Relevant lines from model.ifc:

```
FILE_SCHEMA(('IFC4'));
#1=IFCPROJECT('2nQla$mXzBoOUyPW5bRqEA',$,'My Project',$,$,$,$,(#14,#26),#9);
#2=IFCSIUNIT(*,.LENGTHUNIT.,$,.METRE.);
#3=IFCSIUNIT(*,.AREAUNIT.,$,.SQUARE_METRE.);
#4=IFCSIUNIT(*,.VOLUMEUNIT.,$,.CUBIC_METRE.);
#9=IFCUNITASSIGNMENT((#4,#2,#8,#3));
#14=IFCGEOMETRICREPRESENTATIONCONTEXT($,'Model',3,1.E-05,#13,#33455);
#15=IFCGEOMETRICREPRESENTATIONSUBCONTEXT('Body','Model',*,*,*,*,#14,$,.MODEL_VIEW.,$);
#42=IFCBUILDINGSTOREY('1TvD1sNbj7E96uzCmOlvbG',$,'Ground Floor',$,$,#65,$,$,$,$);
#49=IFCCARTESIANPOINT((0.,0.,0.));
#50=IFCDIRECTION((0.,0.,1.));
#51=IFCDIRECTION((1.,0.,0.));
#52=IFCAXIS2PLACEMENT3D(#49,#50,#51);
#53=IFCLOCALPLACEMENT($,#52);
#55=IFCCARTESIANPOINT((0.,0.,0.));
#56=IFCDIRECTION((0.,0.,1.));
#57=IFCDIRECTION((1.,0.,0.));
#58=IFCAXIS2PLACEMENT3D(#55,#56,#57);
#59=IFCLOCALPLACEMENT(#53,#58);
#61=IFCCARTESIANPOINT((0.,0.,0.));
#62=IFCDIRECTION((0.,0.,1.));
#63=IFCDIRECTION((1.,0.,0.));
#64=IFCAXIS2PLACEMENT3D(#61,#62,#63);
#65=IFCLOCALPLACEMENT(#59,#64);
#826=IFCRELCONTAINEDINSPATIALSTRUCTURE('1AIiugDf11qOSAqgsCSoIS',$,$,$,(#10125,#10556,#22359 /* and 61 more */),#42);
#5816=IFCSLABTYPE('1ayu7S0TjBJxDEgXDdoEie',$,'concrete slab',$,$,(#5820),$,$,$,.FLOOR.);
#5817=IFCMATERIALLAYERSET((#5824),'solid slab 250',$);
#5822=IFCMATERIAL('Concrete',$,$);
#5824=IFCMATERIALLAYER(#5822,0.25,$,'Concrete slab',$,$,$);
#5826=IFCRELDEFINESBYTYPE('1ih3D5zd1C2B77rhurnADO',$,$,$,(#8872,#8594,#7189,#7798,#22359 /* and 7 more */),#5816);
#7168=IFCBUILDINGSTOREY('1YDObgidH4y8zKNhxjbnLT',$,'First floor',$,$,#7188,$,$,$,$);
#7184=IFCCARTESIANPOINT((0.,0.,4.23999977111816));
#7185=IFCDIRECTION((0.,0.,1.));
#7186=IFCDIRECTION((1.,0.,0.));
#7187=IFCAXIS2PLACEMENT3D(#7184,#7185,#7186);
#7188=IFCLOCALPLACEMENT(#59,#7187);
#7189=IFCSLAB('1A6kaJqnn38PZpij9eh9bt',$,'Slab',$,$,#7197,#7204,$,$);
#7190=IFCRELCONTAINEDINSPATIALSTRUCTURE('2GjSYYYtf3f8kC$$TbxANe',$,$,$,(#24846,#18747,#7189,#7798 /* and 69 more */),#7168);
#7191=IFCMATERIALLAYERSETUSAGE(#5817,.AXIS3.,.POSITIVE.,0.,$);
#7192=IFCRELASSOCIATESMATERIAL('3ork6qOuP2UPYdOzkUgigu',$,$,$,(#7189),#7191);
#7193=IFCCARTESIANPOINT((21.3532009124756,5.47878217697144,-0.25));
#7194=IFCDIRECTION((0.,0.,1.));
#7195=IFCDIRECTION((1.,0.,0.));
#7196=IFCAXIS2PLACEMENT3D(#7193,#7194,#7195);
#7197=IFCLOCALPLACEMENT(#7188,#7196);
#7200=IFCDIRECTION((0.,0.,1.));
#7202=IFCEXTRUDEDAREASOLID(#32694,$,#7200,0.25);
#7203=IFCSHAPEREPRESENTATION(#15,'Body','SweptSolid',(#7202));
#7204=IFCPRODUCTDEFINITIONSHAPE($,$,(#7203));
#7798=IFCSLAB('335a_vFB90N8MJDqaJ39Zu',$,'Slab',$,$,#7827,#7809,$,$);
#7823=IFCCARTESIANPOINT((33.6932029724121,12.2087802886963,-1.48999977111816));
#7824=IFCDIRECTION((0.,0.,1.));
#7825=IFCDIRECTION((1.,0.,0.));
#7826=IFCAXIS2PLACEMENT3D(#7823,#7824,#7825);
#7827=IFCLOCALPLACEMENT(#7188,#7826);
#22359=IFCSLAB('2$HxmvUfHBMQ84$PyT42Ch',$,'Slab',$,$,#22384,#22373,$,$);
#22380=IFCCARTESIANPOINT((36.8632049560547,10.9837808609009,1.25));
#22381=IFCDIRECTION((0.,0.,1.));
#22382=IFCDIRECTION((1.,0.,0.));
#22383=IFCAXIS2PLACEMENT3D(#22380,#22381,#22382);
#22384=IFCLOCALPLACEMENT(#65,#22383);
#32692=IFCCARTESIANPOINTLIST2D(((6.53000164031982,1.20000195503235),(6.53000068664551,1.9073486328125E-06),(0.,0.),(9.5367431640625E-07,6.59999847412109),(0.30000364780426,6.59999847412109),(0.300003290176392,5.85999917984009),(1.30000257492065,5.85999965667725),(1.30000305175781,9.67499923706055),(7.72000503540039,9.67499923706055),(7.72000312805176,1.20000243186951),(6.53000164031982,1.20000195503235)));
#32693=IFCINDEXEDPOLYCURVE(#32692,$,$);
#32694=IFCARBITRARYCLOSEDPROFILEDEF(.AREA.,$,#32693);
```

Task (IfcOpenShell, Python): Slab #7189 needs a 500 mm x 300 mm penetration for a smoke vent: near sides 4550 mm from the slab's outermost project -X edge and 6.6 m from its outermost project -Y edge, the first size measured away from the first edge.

```python
import numpy as np
import ifcopenshell
import ifcopenshell.api.feature
import ifcopenshell.api.geometry
import ifcopenshell.api.root
import ifcopenshell.geom
import ifcopenshell.util.placement
import ifcopenshell.util.representation
import ifcopenshell.util.shape
import ifcopenshell.util.unit

model = ifcopenshell.open("model.ifc")
unit_scale = ifcopenshell.util.unit.calculate_unit_scale(model)
settings = ifcopenshell.geom.settings()


def volume(element):
    """Net volume in cubic metres, openings subtracted."""
    shape = ifcopenshell.geom.create_shape(settings, element)
    return ifcopenshell.util.shape.get_volume(shape.geometry)


slab = model.by_guid("1A6kaJqnn38PZpij9eh9bt")
before = volume(slab)

# Extent in the slab's own axes, in metres. The edges named are its -X and -Y sides.
slab_shape = ifcopenshell.geom.create_shape(settings, slab)
vertices = ifcopenshell.util.shape.get_vertices(slab_shape.geometry)
x_min, y_min, bottom = vertices.min(axis=0)
top = vertices[:, 2].max()

opening = ifcopenshell.api.root.create_entity(model, ifc_class="IfcOpeningElement", name="Smoke vent opening", predefined_type="OPENING")
context = ifcopenshell.util.representation.get_context(model, "Model", "Body", "MODEL_VIEW")
width, depth = 0.5, 0.3
outline = [(0.0, 0.0), (width, 0.0), (width, depth), (0.0, depth), (0.0, 0.0)]
# Overshoot both faces by 50 mm so the cut is clean.
shape = ifcopenshell.api.geometry.add_slab_representation(
    model, context=context, depth=top - bottom + 0.1, polyline=outline
)
ifcopenshell.api.geometry.assign_representation(model, product=opening, representation=shape)

matrix = ifcopenshell.util.placement.get_local_placement(slab.ObjectPlacement)
matrix[:, 3] = matrix @ np.append(np.array([x_min + 4.55, y_min + 6.6, bottom - 0.05]) / unit_scale, 1.0)
ifcopenshell.api.geometry.edit_object_placement(model, product=opening, matrix=matrix, is_si=False)
ifcopenshell.api.feature.add_feature(model, feature=opening, element=slab)

after = volume(slab)

print(f"slab volume {before:.3f} -> {after:.3f} m3")

model.write("model_v2.ifc")
```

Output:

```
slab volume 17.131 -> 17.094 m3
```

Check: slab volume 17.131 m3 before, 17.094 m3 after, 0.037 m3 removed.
